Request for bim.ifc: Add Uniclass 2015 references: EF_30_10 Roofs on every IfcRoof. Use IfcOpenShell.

First a look at what the model holds.

```python
import ifcopenshell

model = ifcopenshell.open("bim.ifc")
print(model.schema)
print("classifications:", [c.Name for c in model.by_type("IfcClassification")])
for ifc_class in ("IfcDoor", "IfcRoof", "IfcStair", "IfcWall", "IfcWindow"):
    print(ifc_class, len(model.by_type(ifc_class)))
```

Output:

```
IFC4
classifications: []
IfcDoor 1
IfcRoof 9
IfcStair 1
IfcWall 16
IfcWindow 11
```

```python
import ifcopenshell
import ifcopenshell.api.classification

model = ifcopenshell.open("bim.ifc")

system = ifcopenshell.api.classification.add_classification(model, classification="Uniclass 2015")

codes = {
    "IfcRoof": ("EF_30_10", "Roofs"),
}
for ifc_class, (code, name) in codes.items():
    products = model.by_type(ifc_class)
    ifcopenshell.api.classification.add_reference(
        model, products=products, classification=system, identification=code, name=name
    )
    print(code, len(products))

model.write("bim-out.ifc")
```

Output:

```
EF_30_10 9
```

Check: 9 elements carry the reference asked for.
